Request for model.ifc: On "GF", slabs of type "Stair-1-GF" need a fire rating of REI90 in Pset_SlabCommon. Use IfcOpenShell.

First a look at what the model holds.

```python
import ifcopenshell
import ifcopenshell.util.element

model = ifcopenshell.open("model.ifc")
print(model.schema)
storey = next(s for s in model.by_type("IfcBuildingStorey") if s.Name == "GF")
slabs = [e for e in ifcopenshell.util.element.get_decomposition(storey) if e.is_a("IfcSlab")]
seen = {}
for e in slabs:
    element_type = ifcopenshell.util.element.get_type(e)
    key = (element_type.Name if element_type != e and element_type else None, ifcopenshell.util.element.get_pset(e, "Pset_SlabCommon", "FireRating"))
    seen[key] = seen.get(key, 0) + 1
for (name, value), count in sorted(seen.items(), key=str):
    print(count, "x", name, "|", value)
```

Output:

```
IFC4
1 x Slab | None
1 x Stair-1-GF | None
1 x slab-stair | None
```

```python
import ifcopenshell
import ifcopenshell.api.pset
import ifcopenshell.util.element

model = ifcopenshell.open("model.ifc")

storey = next(s for s in model.by_type("IfcBuildingStorey") if s.Name == "GF")
slabs = [e for e in ifcopenshell.util.element.get_decomposition(storey) if e.is_a("IfcSlab")]

count = 0
for e in slabs:
    element_type = ifcopenshell.util.element.get_type(e)
    if element_type in (None, e) or element_type.Name != "Stair-1-GF":
        continue
    # add_pset returns the element's existing set when there is one.
    pset = ifcopenshell.api.pset.add_pset(model, product=e, name="Pset_SlabCommon")
    ifcopenshell.api.pset.edit_pset(model, pset=pset, properties={"FireRating": "REI90"})
    count += 1

print(count, "slabs updated")

model.write("model_v2.ifc")
```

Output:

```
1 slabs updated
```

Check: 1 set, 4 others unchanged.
